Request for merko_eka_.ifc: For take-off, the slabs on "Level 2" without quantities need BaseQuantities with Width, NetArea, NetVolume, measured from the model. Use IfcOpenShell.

First a look at what the model holds.

```python
import ifcopenshell
import ifcopenshell.util.element
import ifcopenshell.util.unit

model = ifcopenshell.open("merko_eka_.ifc")
print(model.schema)
for unit_type in ("LENGTHUNIT", "AREAUNIT", "VOLUMEUNIT"):
    print(unit_type, ifcopenshell.util.unit.calculate_unit_scale(model, unit_type))
storey = next(s for s in model.by_type("IfcBuildingStorey") if s.Name == "Level 2")
slabs = [e for e in ifcopenshell.util.element.get_decomposition(storey) if e.is_a("IfcSlab")]
for e in sorted(slabs, key=lambda e: e.id()):
    print(e.id(), e.is_a(), e.Name, list(ifcopenshell.util.element.get_psets(e, qtos_only=True)), sep=" | ")
```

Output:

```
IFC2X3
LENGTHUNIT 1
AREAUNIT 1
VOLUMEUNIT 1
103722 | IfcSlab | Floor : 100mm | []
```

```python
import ifcopenshell
import ifcopenshell.api.pset
import ifcopenshell.geom
import ifcopenshell.util.element
import ifcopenshell.util.shape
import ifcopenshell.util.unit

model = ifcopenshell.open("merko_eka_.ifc")
unit_scale = ifcopenshell.util.unit.calculate_unit_scale(model)
area_scale = ifcopenshell.util.unit.calculate_unit_scale(model, "AREAUNIT")
volume_scale = ifcopenshell.util.unit.calculate_unit_scale(model, "VOLUMEUNIT")
settings = ifcopenshell.geom.settings()

storey = next(s for s in model.by_type("IfcBuildingStorey") if s.Name == "Level 2")
slabs = [e for e in ifcopenshell.util.element.get_decomposition(storey) if e.is_a("IfcSlab")]

for e in sorted(slabs, key=lambda e: e.id()):
    if ifcopenshell.util.element.get_psets(e, qtos_only=True, should_inherit=False):
        continue
    # Geometry comes back in metres, in the element's own axes.
    shape = ifcopenshell.geom.create_shape(settings, e)
    values = {
        "Width": ifcopenshell.util.shape.get_z(shape.geometry) / unit_scale,
        "NetArea": ifcopenshell.util.shape.get_footprint_area(shape.geometry) / area_scale,
        "NetVolume": ifcopenshell.util.shape.get_volume(shape.geometry) / volume_scale,
    }
    qto = ifcopenshell.api.pset.add_qto(model, product=e, name="BaseQuantities")
    ifcopenshell.api.pset.edit_qto(model, qto=qto, properties=values)
    print(e.id(), {k: round(v, 3) for k, v in values.items()})

model.write("merko_eka__v2.ifc")
```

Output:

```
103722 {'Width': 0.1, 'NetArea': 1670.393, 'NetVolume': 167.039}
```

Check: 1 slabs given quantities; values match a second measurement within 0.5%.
